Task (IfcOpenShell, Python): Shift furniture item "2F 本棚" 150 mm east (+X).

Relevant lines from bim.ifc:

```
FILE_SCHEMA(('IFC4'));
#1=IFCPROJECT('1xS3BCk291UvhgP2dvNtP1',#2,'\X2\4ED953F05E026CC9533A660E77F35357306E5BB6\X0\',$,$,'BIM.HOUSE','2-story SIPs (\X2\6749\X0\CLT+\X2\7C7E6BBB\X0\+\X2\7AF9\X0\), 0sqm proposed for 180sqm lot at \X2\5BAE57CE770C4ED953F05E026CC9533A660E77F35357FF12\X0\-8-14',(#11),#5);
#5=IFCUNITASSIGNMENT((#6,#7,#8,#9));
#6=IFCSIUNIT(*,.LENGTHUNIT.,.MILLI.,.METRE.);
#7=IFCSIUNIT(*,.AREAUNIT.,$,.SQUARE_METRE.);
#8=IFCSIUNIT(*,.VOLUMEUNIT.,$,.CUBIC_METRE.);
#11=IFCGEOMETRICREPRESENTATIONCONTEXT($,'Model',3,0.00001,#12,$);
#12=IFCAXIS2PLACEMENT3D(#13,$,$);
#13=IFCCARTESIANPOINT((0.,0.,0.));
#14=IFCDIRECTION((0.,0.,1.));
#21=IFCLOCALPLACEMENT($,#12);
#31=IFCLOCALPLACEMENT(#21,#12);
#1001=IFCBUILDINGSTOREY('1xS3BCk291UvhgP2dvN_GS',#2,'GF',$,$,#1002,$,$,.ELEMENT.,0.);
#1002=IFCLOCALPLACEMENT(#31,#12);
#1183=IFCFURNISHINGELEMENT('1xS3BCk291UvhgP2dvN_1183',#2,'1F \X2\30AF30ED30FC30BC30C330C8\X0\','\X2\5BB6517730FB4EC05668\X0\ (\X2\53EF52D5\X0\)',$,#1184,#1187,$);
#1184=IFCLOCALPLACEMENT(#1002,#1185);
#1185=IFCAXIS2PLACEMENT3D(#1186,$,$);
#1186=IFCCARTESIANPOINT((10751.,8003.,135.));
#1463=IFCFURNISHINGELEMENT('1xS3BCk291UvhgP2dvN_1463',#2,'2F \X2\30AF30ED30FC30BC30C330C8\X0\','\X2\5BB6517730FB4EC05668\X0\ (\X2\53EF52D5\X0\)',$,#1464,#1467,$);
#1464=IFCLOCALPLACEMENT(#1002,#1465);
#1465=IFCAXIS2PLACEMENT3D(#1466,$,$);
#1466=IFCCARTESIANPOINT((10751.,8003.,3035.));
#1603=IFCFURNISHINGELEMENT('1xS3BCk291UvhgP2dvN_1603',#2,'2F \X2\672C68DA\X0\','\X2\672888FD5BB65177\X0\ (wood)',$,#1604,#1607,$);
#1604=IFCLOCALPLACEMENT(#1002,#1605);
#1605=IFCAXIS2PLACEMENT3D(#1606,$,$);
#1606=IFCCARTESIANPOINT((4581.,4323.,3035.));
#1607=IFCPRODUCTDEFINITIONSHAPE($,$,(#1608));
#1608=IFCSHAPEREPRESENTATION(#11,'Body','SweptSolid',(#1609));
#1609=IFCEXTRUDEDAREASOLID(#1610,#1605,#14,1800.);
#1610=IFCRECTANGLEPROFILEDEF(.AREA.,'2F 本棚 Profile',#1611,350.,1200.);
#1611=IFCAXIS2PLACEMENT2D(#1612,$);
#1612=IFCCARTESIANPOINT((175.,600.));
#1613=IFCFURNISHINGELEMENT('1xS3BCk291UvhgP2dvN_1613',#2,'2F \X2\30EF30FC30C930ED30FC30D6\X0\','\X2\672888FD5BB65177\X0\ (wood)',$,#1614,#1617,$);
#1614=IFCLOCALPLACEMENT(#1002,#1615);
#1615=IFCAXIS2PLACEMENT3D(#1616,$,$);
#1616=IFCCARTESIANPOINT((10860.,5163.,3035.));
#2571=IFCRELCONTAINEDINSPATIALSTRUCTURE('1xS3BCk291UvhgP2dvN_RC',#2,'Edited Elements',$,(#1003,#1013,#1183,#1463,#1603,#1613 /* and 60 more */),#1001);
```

```python
import ifcopenshell
import ifcopenshell.api.geometry
import ifcopenshell.util.placement
import ifcopenshell.util.unit

model = ifcopenshell.open("bim.ifc")
unit_scale = ifcopenshell.util.unit.calculate_unit_scale(model)

item = model.by_guid("1xS3BCk291UvhgP2dvN_1603")
matrix = ifcopenshell.util.placement.get_local_placement(item.ObjectPlacement)
matrix[0, 3] += 0.15 / unit_scale
ifcopenshell.api.geometry.edit_object_placement(model, product=item, matrix=matrix, is_si=False)

print(ifcopenshell.util.placement.get_local_placement(item.ObjectPlacement).round(3) + 0.0)

model.write("bim-out.ifc")
```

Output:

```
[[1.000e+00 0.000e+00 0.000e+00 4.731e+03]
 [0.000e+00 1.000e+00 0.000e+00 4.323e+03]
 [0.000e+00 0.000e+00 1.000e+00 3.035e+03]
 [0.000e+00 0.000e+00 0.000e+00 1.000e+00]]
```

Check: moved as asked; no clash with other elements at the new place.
